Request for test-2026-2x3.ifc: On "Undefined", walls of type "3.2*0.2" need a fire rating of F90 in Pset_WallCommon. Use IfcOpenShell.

First a look at what the model holds.

```python
import ifcopenshell
import ifcopenshell.util.element

model = ifcopenshell.open("test-2026-2x3.ifc")
print(model.schema)
storey = next(s for s in model.by_type("IfcBuildingStorey") if s.Name == "Undefined")
walls = [e for e in ifcopenshell.util.element.get_decomposition(storey) if e.is_a("IfcWall")]
seen = {}
for e in walls:
    element_type = ifcopenshell.util.element.get_type(e)
    key = (element_type.Name if element_type != e and element_type else None, ifcopenshell.util.element.get_pset(e, "Pset_WallCommon", "FireRating"))
    seen[key] = seen.get(key, 0) + 1
for (name, value), count in sorted(seen.items(), key=str):
    print(count, "x", name, "|", value)
```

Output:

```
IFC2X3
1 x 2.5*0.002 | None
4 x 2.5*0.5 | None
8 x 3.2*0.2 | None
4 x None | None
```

```python
import ifcopenshell
import ifcopenshell.api.pset
import ifcopenshell.util.element

model = ifcopenshell.open("test-2026-2x3.ifc")

storey = next(s for s in model.by_type("IfcBuildingStorey") if s.Name == "Undefined")
walls = [e for e in ifcopenshell.util.element.get_decomposition(storey) if e.is_a("IfcWall")]

count = 0
for e in walls:
    element_type = ifcopenshell.util.element.get_type(e)
    if element_type in (None, e) or element_type.Name != "3.2*0.2":
        continue
    # add_pset returns the element's existing set when there is one.
    pset = ifcopenshell.api.pset.add_pset(model, product=e, name="Pset_WallCommon")
    ifcopenshell.api.pset.edit_pset(model, pset=pset, properties={"FireRating": "F90"})
    count += 1

print(count, "walls updated")

model.write("test-2026-2x3_edited.ifc")
```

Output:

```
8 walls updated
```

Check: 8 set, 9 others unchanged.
